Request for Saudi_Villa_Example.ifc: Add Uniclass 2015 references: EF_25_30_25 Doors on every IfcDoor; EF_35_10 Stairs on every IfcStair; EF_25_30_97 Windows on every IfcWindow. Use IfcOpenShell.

First a look at what the model holds.

```python
import ifcopenshell

model = ifcopenshell.open("Saudi_Villa_Example.ifc")
print(model.schema)
print("classifications:", [c.Name for c in model.by_type("IfcClassification")])
for ifc_class in ("IfcDoor", "IfcRoof", "IfcStair", "IfcWall", "IfcWindow"):
    print(ifc_class, len(model.by_type(ifc_class)))
```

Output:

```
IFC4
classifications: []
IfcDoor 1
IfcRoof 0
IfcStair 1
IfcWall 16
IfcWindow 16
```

```python
import ifcopenshell
import ifcopenshell.api.classification

model = ifcopenshell.open("Saudi_Villa_Example.ifc")

system = ifcopenshell.api.classification.add_classification(model, classification="Uniclass 2015")

codes = {
    "IfcDoor": ("EF_25_30_25", "Doors"),
    "IfcStair": ("EF_35_10", "Stairs"),
    "IfcWindow": ("EF_25_30_97", "Windows"),
}
for ifc_class, (code, name) in codes.items():
    products = model.by_type(ifc_class)
    ifcopenshell.api.classification.add_reference(
        model, products=products, classification=system, identification=code, name=name
    )
    print(code, len(products))

model.write("Saudi_Villa_Example-out.ifc")
```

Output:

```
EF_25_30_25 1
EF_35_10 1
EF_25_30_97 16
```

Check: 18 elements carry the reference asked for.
